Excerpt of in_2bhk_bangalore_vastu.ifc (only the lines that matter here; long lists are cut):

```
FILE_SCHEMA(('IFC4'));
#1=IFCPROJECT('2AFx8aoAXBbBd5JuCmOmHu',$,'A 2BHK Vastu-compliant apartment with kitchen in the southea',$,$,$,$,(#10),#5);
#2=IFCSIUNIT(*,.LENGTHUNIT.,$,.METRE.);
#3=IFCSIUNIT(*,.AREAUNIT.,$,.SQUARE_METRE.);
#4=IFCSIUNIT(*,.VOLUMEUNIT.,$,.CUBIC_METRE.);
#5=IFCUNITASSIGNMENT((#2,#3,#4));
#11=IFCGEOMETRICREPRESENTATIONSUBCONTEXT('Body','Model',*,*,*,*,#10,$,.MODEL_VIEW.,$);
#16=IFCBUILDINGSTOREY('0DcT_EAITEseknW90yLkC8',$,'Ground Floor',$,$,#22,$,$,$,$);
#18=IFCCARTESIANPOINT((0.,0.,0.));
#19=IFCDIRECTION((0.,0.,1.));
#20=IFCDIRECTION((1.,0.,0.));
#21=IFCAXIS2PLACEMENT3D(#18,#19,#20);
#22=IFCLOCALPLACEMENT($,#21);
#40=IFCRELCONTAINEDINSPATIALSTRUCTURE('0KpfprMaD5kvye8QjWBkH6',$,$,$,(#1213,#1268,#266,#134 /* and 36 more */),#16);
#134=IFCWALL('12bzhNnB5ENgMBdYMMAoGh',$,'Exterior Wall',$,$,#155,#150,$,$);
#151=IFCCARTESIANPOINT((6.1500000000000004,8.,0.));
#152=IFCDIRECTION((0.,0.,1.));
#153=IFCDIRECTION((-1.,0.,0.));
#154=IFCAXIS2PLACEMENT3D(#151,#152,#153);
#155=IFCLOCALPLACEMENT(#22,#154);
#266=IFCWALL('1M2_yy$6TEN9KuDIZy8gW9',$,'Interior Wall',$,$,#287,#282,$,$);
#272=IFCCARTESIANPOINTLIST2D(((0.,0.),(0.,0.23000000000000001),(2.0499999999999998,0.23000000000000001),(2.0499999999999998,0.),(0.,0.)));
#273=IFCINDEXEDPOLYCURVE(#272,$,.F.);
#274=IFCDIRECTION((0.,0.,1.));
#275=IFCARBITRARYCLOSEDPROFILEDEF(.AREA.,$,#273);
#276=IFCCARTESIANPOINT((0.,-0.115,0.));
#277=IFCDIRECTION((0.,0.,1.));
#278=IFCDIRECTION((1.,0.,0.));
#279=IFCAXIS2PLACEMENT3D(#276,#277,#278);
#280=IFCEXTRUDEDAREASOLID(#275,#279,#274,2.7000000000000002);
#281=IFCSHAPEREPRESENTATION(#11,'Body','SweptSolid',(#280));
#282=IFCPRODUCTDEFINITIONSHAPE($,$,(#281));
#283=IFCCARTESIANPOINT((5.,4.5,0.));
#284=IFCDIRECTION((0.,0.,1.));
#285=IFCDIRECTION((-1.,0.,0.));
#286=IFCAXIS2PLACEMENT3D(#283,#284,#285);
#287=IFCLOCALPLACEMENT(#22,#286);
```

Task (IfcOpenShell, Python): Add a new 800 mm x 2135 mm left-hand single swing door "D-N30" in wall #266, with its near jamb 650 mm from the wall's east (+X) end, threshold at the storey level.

```python
import numpy as np
import ifcopenshell
import ifcopenshell.api.feature
import ifcopenshell.api.geometry
import ifcopenshell.api.root
import ifcopenshell.api.spatial
import ifcopenshell.geom
import ifcopenshell.util.element
import ifcopenshell.util.placement
import ifcopenshell.util.representation
import ifcopenshell.util.shape
import ifcopenshell.util.unit

model = ifcopenshell.open("in_2bhk_bangalore_vastu.ifc")
unit_scale = ifcopenshell.util.unit.calculate_unit_scale(model)
settings = ifcopenshell.geom.settings()


def volume(element):
    """Net volume in cubic metres, openings subtracted."""
    shape = ifcopenshell.geom.create_shape(settings, element)
    return ifcopenshell.util.shape.get_volume(shape.geometry)


wall = model.by_id(266)
storey = ifcopenshell.util.element.get_container(wall, ifc_class="IfcBuildingStorey")
context = ifcopenshell.util.representation.get_context(model, "Model", "Body", "MODEL_VIEW")
before = volume(wall)

width, height, from_end, sill = 0.8, 2.135, 0.65, 0.0  # metres

# The wall runs along its own X axis, and the end named is its -X end.
wall_shape = ifcopenshell.geom.create_shape(settings, wall)
x, y, z = ifcopenshell.util.shape.get_vertices(wall_shape.geometry).T
start = x.min() + from_end
face, thickness = float(y.min()), float(y.max() - y.min())
wall_matrix = ifcopenshell.util.placement.get_local_placement(wall.ObjectPlacement)
level = ifcopenshell.util.placement.get_local_placement(storey.ObjectPlacement)[2, 3]


def in_wall(x, y):
    """Placement at x, y metres in the wall's axes, at sill height."""
    matrix = wall_matrix.copy()
    matrix[:, 3] = wall_matrix @ np.array([x / unit_scale, y / unit_scale, 0.0, 1.0])
    matrix[2, 3] = level + sill / unit_scale
    return matrix


# Opening: a box that overshoots both wall faces by 50 mm.
opening = ifcopenshell.api.root.create_entity(model, ifc_class="IfcOpeningElement", predefined_type="OPENING")
box = ifcopenshell.api.geometry.add_wall_representation(
    model, context=context, length=width, height=height, thickness=thickness + 0.1
)
ifcopenshell.api.geometry.assign_representation(model, product=opening, representation=box)
ifcopenshell.api.geometry.edit_object_placement(model, product=opening, matrix=in_wall(start, face - 0.05), is_si=False)
ifcopenshell.api.feature.add_feature(model, feature=opening, element=wall)

door = ifcopenshell.api.root.create_entity(model, ifc_class="IfcDoor", name="D-N30", predefined_type="DOOR")
door.OverallWidth, door.OverallHeight = width / unit_scale, height / unit_scale
door.OperationType = "SINGLE_SWING_LEFT"
body = ifcopenshell.api.geometry.add_door_representation(
    model,
    context=context,
    overall_width=door.OverallWidth,
    overall_height=door.OverallHeight,
    operation_type="SINGLE_SWING_LEFT",
    lining_properties={"LiningDepth": thickness / unit_scale, "ThresholdDepth": thickness / unit_scale},
)
ifcopenshell.api.geometry.assign_representation(model, product=door, representation=body)
ifcopenshell.api.spatial.assign_container(model, products=[door], relating_structure=storey)
ifcopenshell.api.feature.add_filling(model, opening=opening, element=door)

# The lining spans the wall, so the door starts at the wall face.
ifcopenshell.api.geometry.edit_object_placement(model, product=door, matrix=in_wall(start, face), is_si=False)

after = volume(wall)

print(f"wall volume {before:.3f} -> {after:.3f} m3")

model.write("in_2bhk_bangalore_vastu_edited.ifc")
```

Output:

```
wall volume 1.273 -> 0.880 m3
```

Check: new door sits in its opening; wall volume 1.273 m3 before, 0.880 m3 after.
